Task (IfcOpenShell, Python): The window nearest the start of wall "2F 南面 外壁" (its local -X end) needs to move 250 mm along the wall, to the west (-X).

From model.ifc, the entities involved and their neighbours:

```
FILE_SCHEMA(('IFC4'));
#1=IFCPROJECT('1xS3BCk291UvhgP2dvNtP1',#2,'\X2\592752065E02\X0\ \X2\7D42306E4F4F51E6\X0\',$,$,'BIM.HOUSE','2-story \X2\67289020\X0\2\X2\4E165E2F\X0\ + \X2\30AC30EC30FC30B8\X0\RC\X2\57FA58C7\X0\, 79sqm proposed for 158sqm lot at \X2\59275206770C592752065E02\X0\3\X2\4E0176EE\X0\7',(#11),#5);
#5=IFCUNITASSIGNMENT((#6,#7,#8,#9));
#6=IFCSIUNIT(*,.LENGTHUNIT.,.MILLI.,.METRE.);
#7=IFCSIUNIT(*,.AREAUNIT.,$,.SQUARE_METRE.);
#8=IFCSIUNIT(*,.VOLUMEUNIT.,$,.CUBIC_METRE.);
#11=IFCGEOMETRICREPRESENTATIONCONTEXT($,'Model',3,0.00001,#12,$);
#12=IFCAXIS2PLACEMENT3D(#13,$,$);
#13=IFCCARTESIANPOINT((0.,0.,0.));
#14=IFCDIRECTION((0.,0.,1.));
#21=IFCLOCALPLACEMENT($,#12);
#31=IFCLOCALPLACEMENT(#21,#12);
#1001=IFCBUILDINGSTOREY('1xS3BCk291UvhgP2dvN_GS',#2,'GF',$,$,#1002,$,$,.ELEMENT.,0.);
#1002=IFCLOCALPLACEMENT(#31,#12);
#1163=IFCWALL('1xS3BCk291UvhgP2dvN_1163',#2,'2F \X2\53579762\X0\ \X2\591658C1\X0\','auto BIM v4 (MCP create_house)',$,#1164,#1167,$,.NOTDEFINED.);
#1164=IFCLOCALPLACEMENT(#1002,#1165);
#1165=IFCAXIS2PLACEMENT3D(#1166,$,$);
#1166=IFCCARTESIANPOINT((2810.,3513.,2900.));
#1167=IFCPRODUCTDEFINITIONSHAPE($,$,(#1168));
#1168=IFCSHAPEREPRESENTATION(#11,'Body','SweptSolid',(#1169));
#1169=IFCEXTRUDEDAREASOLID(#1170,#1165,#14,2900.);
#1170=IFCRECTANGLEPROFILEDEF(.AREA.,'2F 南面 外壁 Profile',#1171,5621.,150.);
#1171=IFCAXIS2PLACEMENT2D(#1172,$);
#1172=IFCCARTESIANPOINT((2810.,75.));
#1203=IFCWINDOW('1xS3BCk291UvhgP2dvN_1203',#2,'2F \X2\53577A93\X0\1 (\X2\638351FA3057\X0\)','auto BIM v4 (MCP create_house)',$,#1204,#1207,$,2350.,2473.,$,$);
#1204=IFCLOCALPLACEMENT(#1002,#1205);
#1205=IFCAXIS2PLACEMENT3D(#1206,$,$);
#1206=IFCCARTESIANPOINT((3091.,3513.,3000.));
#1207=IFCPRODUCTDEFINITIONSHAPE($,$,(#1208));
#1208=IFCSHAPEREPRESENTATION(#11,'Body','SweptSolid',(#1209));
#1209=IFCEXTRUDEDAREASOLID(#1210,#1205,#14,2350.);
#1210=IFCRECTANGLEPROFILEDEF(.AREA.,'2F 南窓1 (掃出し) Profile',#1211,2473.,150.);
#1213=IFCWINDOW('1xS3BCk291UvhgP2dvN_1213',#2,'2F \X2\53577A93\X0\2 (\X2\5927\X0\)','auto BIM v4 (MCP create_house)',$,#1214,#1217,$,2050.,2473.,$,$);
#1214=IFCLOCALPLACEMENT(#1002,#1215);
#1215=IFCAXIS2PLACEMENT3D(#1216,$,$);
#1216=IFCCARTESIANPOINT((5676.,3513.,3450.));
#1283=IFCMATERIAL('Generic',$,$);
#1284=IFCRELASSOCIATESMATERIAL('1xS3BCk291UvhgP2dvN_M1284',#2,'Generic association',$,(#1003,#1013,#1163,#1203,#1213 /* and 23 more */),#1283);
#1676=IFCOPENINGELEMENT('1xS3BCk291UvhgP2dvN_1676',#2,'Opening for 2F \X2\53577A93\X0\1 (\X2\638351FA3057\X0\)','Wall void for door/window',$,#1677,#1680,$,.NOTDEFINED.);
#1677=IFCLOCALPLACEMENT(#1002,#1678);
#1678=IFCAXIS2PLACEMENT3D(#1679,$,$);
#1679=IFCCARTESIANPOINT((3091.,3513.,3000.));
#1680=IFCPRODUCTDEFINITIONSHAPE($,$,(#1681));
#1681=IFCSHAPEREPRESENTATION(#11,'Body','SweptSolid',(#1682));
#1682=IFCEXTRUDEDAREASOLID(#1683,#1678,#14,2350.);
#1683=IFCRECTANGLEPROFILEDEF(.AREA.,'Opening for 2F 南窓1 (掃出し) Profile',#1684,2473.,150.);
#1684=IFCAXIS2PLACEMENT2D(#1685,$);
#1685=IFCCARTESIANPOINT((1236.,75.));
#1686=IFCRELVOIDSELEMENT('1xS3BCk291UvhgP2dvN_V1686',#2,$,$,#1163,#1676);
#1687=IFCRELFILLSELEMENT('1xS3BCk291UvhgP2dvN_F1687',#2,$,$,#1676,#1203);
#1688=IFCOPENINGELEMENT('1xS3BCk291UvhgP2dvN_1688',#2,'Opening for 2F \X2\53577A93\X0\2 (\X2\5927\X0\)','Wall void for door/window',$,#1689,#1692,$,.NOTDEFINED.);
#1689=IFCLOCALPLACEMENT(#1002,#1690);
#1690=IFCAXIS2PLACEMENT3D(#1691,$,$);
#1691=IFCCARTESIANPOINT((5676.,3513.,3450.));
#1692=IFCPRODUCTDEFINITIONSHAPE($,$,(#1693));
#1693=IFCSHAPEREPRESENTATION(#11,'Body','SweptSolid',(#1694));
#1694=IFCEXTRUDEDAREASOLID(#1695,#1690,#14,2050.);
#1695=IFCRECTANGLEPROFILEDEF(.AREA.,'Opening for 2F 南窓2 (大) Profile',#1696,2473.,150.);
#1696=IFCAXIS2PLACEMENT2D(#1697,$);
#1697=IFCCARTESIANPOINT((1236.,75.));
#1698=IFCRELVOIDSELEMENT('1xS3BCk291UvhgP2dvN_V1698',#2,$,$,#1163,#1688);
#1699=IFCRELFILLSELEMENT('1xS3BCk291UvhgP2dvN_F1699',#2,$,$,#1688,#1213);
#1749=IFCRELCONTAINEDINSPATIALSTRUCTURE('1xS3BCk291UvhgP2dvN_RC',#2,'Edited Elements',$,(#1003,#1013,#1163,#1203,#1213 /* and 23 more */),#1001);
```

```python
import ifcopenshell
import ifcopenshell.api.geometry
import ifcopenshell.util.placement
import ifcopenshell.util.unit

model = ifcopenshell.open("model.ifc")
unit_scale = ifcopenshell.util.unit.calculate_unit_scale(model)

window = model.by_guid("1xS3BCk291UvhgP2dvN_1203")
opening = window.FillsVoids[0].RelatingOpeningElement
wall = opening.VoidsElements[0].RelatingBuildingElement

wall_matrix = ifcopenshell.util.placement.get_local_placement(wall.ObjectPlacement)
shift = wall_matrix[:3, 0] * -0.25 / unit_scale
before = ifcopenshell.util.placement.get_local_placement(window.ObjectPlacement)[:3, 3].copy()

# The window is not placed relative to its opening, so move both.
for product in (opening, window):
    matrix = ifcopenshell.util.placement.get_local_placement(product.ObjectPlacement)
    matrix[:3, 3] += shift
    ifcopenshell.api.geometry.edit_object_placement(model, product=product, matrix=matrix, is_si=False)

after = ifcopenshell.util.placement.get_local_placement(window.ObjectPlacement)[:3, 3]
print("window moved by", (after - before).round(3) + 0.0)

model.write("model-out.ifc")
```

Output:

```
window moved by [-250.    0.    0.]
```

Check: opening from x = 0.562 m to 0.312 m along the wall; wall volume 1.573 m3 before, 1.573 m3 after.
